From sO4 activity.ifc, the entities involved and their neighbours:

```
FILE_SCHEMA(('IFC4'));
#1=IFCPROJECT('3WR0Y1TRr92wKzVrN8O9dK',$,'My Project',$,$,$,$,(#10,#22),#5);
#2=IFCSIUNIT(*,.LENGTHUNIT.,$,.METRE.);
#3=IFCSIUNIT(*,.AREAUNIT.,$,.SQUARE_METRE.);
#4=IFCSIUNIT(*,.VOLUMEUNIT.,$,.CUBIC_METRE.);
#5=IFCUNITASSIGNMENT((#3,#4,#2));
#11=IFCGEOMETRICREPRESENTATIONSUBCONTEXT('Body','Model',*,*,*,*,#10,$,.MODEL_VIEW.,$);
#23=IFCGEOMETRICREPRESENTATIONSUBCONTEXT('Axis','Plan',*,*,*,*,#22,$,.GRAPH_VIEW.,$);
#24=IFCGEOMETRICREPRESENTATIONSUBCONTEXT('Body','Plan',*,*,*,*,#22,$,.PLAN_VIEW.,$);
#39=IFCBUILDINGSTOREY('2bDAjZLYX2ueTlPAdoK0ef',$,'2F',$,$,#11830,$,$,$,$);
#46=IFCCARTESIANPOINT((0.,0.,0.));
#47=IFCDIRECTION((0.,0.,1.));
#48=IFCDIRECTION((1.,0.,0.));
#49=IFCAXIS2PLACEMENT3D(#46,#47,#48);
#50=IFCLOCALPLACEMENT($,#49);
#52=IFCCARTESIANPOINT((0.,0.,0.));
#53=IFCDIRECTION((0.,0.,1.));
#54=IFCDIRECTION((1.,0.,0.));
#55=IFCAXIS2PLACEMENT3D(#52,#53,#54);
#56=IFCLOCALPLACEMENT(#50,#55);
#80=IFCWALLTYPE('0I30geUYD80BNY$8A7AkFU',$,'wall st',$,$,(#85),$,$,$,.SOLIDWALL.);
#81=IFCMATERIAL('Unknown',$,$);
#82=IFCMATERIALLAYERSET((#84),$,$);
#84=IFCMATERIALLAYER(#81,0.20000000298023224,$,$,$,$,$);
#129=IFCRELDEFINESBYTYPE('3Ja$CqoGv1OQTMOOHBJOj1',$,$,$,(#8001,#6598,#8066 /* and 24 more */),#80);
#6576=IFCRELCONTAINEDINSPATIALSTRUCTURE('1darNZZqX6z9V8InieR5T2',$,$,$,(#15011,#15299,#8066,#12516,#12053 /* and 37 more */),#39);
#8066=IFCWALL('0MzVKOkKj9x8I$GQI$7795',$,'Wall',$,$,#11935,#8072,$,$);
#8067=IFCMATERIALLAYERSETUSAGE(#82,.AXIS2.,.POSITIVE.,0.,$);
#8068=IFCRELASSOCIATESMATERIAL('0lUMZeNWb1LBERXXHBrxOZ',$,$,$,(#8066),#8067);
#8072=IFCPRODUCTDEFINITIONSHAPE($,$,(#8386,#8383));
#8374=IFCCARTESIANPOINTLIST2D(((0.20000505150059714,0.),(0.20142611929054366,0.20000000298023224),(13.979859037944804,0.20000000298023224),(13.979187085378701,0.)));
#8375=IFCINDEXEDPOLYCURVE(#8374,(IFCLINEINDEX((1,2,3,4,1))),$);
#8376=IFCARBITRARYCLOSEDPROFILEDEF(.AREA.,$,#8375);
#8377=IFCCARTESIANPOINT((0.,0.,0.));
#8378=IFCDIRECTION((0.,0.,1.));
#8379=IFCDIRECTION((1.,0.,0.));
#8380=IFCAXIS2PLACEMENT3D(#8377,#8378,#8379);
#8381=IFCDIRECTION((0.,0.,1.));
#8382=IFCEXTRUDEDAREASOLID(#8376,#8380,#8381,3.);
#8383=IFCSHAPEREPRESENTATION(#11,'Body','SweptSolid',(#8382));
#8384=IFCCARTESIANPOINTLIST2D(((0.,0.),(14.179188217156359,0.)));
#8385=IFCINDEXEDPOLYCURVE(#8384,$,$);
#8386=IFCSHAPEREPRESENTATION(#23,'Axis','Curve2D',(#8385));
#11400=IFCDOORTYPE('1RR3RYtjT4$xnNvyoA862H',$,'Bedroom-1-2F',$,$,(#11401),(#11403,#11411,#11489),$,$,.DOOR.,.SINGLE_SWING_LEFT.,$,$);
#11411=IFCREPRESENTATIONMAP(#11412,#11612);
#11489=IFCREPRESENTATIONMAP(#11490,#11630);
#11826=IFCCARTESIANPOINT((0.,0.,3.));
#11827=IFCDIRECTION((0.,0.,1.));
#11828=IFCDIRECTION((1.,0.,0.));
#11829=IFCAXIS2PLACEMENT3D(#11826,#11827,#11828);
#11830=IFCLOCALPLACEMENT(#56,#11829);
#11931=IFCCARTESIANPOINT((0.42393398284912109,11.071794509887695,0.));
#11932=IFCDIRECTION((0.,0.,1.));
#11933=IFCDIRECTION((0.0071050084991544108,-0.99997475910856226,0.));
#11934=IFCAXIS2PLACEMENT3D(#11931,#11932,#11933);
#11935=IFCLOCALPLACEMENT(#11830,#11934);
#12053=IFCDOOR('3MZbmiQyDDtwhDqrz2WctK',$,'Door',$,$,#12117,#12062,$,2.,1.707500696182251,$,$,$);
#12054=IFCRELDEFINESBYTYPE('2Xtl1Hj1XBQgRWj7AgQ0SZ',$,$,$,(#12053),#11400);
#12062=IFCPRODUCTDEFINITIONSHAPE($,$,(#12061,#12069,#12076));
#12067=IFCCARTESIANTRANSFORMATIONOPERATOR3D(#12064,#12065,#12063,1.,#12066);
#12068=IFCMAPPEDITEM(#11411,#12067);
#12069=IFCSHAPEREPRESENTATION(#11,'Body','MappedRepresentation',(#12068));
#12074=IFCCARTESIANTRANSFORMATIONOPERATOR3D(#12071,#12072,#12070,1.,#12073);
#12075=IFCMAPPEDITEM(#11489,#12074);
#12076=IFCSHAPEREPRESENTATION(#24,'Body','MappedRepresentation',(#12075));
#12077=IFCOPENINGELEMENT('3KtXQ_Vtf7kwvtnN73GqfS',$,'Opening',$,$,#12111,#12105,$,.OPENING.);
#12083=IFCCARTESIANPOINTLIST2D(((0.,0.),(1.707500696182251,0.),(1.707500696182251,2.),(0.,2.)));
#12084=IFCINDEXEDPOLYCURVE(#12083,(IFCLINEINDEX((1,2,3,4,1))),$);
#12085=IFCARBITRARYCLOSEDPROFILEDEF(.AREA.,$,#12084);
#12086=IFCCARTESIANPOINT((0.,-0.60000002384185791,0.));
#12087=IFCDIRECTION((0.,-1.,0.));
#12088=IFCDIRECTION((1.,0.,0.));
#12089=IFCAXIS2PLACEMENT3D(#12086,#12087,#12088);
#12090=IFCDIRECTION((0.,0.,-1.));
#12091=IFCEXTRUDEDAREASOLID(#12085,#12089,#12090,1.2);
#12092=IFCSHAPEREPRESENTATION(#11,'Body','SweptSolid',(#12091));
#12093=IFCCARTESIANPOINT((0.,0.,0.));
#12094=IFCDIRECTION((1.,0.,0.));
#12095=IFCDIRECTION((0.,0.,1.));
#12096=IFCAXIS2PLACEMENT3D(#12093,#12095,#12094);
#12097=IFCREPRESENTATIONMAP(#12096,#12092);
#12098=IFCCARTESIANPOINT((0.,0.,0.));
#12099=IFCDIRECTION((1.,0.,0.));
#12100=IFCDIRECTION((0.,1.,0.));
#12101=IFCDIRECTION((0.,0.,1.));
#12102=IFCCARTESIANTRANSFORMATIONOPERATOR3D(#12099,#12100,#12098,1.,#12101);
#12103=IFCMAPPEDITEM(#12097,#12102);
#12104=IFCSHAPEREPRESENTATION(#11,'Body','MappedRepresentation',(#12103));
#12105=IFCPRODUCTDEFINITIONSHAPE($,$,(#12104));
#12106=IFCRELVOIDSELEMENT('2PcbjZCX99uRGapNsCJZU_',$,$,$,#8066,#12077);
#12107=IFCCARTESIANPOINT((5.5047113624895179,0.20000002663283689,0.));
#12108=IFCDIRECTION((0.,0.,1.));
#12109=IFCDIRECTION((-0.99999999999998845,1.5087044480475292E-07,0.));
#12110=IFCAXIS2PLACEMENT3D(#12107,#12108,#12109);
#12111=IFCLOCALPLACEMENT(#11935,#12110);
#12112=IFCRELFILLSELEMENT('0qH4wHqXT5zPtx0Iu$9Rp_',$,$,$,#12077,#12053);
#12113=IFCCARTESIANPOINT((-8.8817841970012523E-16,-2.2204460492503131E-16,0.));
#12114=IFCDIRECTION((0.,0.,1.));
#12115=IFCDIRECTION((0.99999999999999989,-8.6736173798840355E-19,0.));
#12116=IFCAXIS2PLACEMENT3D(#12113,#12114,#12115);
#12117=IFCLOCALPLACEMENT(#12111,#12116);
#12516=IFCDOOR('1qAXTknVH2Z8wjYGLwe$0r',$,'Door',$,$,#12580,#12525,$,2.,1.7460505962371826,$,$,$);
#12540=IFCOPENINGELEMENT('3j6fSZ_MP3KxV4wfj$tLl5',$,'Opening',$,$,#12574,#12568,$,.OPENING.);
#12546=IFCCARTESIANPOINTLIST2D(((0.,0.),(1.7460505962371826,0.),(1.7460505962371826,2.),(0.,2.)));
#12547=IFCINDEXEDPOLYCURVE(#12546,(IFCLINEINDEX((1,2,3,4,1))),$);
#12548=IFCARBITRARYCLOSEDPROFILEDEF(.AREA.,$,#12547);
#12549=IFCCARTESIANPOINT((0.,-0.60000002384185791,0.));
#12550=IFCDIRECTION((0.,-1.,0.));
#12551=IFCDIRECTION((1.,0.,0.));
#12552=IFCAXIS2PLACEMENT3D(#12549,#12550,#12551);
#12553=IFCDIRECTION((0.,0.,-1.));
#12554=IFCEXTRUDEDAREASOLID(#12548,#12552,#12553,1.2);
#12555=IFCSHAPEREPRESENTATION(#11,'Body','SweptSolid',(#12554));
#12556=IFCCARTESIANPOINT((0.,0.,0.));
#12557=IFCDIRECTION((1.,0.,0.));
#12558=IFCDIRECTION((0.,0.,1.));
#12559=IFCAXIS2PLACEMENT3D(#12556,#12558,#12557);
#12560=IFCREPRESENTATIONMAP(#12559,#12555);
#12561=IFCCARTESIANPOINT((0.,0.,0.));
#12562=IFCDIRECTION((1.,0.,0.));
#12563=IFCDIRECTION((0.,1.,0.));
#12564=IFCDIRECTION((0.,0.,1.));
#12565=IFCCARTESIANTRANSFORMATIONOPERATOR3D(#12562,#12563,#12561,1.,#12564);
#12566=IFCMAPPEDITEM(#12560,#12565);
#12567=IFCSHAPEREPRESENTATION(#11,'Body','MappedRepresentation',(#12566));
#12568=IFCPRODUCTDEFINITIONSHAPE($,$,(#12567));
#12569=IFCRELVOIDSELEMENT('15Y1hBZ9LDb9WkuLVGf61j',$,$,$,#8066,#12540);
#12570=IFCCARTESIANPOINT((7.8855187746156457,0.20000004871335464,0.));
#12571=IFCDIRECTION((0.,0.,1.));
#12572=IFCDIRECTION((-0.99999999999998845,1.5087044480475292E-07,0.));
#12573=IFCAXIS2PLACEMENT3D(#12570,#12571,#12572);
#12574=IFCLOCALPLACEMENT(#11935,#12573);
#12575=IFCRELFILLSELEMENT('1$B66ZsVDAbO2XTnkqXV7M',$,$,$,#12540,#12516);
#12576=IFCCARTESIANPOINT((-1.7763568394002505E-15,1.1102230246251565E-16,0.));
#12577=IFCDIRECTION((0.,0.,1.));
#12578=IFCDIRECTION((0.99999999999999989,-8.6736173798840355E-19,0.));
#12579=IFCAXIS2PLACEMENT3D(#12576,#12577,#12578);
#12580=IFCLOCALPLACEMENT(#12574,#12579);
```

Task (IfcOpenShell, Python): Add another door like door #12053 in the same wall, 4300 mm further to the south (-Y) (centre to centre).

```python
import ifcopenshell
import ifcopenshell.api.feature
import ifcopenshell.api.geometry
import ifcopenshell.api.root
import ifcopenshell.geom
import ifcopenshell.util.element
import ifcopenshell.util.placement
import ifcopenshell.util.shape

model = ifcopenshell.open("sO4 activity.ifc")
settings = ifcopenshell.geom.settings()


def volume(element):
    """Net volume in cubic metres, openings subtracted."""
    shape = ifcopenshell.geom.create_shape(settings, element)
    return ifcopenshell.util.shape.get_volume(shape.geometry)


door = model.by_guid("3MZbmiQyDDtwhDqrz2WctK")
opening = door.FillsVoids[0].RelatingOpeningElement
wall = opening.VoidsElements[0].RelatingBuildingElement
before = volume(wall)
shift = ifcopenshell.util.placement.get_local_placement(wall.ObjectPlacement)[:3, 0] * 4.3

# copy_class copies the void relationship, type, container and properties, but no geometry.
new_opening = ifcopenshell.api.root.copy_class(model, product=opening)
new_opening.Representation = ifcopenshell.util.element.copy_deep(
    model, opening.Representation, exclude=["IfcGeometricRepresentationContext", "IfcRepresentationMap"]
)
new_door = ifcopenshell.api.root.copy_class(model, product=door)
new_door.Representation = ifcopenshell.util.element.copy_deep(
    model, door.Representation, exclude=["IfcGeometricRepresentationContext", "IfcRepresentationMap"]
)
ifcopenshell.api.feature.add_filling(model, opening=new_opening, element=new_door)

for old, new in ((opening, new_opening), (door, new_door)):
    matrix = ifcopenshell.util.placement.get_local_placement(old.ObjectPlacement)
    matrix[:3, 3] += shift
    ifcopenshell.api.geometry.edit_object_placement(model, product=new, matrix=matrix, is_si=False)

after = volume(wall)

print(f"wall volume {before:.3f} -> {after:.3f} m3")

model.write("sO4 activity_v2.ifc")
```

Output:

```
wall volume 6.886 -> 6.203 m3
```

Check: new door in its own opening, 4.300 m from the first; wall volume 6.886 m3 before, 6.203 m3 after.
